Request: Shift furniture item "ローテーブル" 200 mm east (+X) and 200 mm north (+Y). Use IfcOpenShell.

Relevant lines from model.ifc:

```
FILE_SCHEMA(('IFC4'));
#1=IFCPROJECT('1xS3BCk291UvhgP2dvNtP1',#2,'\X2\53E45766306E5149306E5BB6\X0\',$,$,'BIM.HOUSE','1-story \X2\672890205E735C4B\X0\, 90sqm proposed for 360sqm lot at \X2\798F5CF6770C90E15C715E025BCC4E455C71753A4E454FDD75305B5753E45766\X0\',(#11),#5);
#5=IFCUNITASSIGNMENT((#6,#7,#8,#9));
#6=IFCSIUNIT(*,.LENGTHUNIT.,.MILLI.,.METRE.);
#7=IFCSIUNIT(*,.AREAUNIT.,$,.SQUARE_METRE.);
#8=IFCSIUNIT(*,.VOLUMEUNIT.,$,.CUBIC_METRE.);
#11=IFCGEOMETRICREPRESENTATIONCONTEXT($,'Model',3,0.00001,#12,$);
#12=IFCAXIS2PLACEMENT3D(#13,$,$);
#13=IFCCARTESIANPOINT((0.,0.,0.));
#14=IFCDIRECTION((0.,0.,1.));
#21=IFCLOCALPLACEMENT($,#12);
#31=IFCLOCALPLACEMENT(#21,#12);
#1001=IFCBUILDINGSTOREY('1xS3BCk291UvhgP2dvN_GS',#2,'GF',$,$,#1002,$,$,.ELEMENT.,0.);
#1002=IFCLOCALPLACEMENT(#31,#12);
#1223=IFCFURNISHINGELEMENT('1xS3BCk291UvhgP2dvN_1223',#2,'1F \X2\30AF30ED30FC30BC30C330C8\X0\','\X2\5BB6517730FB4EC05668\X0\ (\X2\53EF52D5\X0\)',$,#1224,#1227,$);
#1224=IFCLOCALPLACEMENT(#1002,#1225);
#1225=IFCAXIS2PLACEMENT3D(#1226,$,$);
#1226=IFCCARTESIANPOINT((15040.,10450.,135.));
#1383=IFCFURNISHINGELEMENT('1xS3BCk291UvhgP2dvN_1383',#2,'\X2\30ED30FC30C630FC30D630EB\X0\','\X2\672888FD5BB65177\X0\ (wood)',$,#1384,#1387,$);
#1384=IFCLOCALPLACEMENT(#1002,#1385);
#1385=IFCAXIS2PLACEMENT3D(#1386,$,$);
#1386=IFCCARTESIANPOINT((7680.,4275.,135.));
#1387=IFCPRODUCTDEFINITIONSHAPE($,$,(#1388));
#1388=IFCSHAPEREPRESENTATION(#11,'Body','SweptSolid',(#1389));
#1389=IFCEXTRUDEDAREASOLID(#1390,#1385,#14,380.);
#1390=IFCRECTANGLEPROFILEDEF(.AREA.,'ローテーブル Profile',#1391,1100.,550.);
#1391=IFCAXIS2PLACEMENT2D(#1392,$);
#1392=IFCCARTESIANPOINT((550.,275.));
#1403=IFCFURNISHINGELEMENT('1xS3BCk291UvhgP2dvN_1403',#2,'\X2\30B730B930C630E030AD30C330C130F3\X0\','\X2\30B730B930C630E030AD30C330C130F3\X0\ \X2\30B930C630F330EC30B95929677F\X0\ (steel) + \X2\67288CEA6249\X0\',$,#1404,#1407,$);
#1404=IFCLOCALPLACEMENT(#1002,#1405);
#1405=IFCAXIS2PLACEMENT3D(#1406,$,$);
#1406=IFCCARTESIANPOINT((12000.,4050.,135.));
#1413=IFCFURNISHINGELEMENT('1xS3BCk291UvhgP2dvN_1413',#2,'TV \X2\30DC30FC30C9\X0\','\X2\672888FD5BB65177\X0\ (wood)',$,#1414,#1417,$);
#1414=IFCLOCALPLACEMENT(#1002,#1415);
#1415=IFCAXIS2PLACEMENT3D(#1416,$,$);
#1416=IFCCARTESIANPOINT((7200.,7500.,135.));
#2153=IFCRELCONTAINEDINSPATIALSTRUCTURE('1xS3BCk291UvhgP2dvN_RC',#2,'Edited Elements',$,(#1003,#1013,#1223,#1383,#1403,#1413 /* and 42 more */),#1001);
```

```python
import ifcopenshell
import ifcopenshell.api.geometry
import ifcopenshell.util.placement
import ifcopenshell.util.unit

model = ifcopenshell.open("model.ifc")
unit_scale = ifcopenshell.util.unit.calculate_unit_scale(model)

item = model.by_id(1383)
matrix = ifcopenshell.util.placement.get_local_placement(item.ObjectPlacement)
matrix[0, 3] += 0.2 / unit_scale
matrix[1, 3] += 0.2 / unit_scale
ifcopenshell.api.geometry.edit_object_placement(model, product=item, matrix=matrix, is_si=False)

print(ifcopenshell.util.placement.get_local_placement(item.ObjectPlacement).round(3) + 0.0)

model.write("model_v2.ifc")
```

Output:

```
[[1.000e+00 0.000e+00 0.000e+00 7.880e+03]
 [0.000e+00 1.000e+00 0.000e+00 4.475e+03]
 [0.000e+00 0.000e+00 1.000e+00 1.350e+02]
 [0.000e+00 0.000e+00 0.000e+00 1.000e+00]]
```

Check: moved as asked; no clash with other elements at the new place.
